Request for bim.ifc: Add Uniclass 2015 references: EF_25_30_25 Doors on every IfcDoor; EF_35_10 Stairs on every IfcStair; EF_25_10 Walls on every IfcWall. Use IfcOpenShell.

First a look at what the model holds.

```python
import ifcopenshell

model = ifcopenshell.open("bim.ifc")
print(model.schema)
print("classifications:", [c.Name for c in model.by_type("IfcClassification")])
for ifc_class in ("IfcDoor", "IfcRoof", "IfcStair", "IfcWall", "IfcWindow"):
    print(ifc_class, len(model.by_type(ifc_class)))
```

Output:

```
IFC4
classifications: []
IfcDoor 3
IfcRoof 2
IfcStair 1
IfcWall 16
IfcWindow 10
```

```python
import ifcopenshell
import ifcopenshell.api.classification

model = ifcopenshell.open("bim.ifc")

system = ifcopenshell.api.classification.add_classification(model, classification="Uniclass 2015")

codes = {
    "IfcDoor": ("EF_25_30_25", "Doors"),
    "IfcStair": ("EF_35_10", "Stairs"),
    "IfcWall": ("EF_25_10", "Walls"),
}
for ifc_class, (code, name) in codes.items():
    products = model.by_type(ifc_class)
    ifcopenshell.api.classification.add_reference(
        model, products=products, classification=system, identification=code, name=name
    )
    print(code, len(products))

model.write("bim_v2.ifc")
```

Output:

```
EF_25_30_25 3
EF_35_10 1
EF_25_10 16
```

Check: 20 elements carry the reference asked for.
